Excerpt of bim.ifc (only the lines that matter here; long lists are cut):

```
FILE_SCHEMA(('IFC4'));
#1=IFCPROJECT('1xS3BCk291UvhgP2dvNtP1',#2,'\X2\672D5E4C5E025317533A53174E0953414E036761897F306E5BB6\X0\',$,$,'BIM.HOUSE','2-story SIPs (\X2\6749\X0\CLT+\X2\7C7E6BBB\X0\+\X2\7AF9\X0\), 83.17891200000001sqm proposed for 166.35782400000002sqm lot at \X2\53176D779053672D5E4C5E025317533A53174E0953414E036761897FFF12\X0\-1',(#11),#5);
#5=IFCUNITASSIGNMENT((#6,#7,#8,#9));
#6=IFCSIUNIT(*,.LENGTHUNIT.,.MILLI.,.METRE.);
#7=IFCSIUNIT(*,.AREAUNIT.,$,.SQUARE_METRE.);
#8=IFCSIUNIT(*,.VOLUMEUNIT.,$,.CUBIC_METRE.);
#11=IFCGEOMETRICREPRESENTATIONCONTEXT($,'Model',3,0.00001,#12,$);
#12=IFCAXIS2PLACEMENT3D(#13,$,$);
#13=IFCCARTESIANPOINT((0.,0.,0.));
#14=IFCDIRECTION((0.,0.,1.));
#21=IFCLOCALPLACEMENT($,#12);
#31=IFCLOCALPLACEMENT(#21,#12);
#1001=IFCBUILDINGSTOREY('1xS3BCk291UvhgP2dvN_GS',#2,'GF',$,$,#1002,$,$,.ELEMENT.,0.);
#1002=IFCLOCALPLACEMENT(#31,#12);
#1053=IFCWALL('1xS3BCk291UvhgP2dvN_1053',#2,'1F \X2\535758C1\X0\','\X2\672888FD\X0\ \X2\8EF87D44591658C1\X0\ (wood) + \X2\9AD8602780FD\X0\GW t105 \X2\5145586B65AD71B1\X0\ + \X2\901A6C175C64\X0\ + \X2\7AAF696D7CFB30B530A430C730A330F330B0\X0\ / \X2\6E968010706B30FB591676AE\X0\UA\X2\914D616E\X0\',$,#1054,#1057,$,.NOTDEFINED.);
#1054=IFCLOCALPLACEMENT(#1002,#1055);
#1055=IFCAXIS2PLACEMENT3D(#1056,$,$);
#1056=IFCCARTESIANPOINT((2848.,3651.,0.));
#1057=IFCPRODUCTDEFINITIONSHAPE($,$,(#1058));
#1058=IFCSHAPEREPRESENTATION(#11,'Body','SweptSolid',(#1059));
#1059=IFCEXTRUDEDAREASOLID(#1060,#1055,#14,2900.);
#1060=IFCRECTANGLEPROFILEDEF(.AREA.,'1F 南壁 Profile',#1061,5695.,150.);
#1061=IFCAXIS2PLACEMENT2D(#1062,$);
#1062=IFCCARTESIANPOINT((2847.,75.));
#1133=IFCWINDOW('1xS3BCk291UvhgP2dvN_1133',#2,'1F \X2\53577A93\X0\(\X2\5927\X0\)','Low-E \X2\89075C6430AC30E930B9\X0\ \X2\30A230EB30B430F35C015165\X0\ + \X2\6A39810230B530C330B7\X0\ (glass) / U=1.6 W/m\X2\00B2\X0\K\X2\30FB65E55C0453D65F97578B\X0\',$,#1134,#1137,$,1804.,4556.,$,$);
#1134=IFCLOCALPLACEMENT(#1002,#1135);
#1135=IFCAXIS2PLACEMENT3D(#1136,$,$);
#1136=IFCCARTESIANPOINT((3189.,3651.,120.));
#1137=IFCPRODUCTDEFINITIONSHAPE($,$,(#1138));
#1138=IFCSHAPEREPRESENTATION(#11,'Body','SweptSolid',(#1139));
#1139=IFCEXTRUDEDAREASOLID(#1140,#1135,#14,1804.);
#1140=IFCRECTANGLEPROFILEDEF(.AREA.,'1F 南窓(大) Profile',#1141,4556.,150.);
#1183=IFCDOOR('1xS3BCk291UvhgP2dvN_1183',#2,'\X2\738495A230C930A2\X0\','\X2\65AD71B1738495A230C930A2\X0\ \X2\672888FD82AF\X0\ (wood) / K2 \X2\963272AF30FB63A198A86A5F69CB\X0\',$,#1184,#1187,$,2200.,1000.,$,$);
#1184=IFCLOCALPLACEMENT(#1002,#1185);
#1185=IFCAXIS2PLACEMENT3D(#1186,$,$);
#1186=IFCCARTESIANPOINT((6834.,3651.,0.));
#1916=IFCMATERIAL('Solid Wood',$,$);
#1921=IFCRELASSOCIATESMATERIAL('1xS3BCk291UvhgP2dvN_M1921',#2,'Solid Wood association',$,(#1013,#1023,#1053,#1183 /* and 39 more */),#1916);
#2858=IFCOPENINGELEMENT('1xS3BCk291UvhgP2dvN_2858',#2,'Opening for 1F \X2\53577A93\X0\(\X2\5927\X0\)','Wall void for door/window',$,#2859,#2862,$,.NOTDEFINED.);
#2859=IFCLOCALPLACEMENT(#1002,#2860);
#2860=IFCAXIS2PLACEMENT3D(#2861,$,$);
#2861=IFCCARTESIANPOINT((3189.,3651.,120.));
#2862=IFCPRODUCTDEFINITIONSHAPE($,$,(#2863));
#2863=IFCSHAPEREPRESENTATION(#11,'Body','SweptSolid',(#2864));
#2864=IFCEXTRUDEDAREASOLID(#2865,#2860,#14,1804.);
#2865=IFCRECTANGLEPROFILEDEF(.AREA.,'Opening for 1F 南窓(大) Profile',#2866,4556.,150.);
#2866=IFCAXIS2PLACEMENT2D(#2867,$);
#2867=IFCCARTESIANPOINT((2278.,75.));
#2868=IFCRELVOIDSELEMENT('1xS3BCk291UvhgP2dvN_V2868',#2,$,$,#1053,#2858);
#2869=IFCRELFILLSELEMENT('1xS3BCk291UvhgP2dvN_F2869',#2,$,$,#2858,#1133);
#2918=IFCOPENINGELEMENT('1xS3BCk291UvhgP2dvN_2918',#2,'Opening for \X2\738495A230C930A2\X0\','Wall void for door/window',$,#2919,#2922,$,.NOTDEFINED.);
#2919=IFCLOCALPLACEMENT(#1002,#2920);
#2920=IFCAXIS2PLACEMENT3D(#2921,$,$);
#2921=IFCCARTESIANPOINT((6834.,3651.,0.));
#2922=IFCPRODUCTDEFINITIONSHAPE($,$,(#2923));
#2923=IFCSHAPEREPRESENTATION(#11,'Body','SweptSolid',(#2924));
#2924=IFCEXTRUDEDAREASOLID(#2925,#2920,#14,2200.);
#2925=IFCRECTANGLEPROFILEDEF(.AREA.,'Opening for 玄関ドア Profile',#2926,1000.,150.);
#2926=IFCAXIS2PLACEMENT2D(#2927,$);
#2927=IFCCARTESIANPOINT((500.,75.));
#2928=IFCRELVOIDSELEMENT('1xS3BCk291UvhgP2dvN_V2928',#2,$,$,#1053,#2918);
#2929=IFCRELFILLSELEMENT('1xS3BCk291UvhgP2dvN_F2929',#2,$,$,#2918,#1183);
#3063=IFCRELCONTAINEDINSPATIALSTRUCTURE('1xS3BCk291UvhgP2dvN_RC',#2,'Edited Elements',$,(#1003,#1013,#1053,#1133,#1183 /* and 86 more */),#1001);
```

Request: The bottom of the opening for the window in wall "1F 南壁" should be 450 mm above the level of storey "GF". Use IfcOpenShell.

```python
import numpy as np
import ifcopenshell
import ifcopenshell.api.geometry
import ifcopenshell.geom
import ifcopenshell.util.element
import ifcopenshell.util.placement
import ifcopenshell.util.shape
import ifcopenshell.util.unit

model = ifcopenshell.open("bim.ifc")
unit_scale = ifcopenshell.util.unit.calculate_unit_scale(model)

window = model.by_guid("1xS3BCk291UvhgP2dvN_1133")
opening = window.FillsVoids[0].RelatingOpeningElement
storey = ifcopenshell.util.element.get_container(window, ifc_class="IfcBuildingStorey")
level = ifcopenshell.util.placement.get_local_placement(storey.ObjectPlacement)[2, 3]

# The opening's origin need not be at the sill, so measure its lowest point.
shape = ifcopenshell.geom.create_shape(ifcopenshell.geom.settings(), opening)
bottom = ifcopenshell.util.shape.get_shape_bottom_elevation(shape, shape.geometry) / unit_scale
dz = level + 450.0 - bottom

shift = np.array([0.0, 0.0, dz])
# The window is not placed relative to its opening, so move both.
for product in (opening, window):
    matrix = ifcopenshell.util.placement.get_local_placement(product.ObjectPlacement)
    matrix[:3, 3] += shift
    ifcopenshell.api.geometry.edit_object_placement(model, product=product, matrix=matrix, is_si=False)

print(f"moved by {dz * unit_scale:+.3f} m")

model.write("bim_updated.ifc")
```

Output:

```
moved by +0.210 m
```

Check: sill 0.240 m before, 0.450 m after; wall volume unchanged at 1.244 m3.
